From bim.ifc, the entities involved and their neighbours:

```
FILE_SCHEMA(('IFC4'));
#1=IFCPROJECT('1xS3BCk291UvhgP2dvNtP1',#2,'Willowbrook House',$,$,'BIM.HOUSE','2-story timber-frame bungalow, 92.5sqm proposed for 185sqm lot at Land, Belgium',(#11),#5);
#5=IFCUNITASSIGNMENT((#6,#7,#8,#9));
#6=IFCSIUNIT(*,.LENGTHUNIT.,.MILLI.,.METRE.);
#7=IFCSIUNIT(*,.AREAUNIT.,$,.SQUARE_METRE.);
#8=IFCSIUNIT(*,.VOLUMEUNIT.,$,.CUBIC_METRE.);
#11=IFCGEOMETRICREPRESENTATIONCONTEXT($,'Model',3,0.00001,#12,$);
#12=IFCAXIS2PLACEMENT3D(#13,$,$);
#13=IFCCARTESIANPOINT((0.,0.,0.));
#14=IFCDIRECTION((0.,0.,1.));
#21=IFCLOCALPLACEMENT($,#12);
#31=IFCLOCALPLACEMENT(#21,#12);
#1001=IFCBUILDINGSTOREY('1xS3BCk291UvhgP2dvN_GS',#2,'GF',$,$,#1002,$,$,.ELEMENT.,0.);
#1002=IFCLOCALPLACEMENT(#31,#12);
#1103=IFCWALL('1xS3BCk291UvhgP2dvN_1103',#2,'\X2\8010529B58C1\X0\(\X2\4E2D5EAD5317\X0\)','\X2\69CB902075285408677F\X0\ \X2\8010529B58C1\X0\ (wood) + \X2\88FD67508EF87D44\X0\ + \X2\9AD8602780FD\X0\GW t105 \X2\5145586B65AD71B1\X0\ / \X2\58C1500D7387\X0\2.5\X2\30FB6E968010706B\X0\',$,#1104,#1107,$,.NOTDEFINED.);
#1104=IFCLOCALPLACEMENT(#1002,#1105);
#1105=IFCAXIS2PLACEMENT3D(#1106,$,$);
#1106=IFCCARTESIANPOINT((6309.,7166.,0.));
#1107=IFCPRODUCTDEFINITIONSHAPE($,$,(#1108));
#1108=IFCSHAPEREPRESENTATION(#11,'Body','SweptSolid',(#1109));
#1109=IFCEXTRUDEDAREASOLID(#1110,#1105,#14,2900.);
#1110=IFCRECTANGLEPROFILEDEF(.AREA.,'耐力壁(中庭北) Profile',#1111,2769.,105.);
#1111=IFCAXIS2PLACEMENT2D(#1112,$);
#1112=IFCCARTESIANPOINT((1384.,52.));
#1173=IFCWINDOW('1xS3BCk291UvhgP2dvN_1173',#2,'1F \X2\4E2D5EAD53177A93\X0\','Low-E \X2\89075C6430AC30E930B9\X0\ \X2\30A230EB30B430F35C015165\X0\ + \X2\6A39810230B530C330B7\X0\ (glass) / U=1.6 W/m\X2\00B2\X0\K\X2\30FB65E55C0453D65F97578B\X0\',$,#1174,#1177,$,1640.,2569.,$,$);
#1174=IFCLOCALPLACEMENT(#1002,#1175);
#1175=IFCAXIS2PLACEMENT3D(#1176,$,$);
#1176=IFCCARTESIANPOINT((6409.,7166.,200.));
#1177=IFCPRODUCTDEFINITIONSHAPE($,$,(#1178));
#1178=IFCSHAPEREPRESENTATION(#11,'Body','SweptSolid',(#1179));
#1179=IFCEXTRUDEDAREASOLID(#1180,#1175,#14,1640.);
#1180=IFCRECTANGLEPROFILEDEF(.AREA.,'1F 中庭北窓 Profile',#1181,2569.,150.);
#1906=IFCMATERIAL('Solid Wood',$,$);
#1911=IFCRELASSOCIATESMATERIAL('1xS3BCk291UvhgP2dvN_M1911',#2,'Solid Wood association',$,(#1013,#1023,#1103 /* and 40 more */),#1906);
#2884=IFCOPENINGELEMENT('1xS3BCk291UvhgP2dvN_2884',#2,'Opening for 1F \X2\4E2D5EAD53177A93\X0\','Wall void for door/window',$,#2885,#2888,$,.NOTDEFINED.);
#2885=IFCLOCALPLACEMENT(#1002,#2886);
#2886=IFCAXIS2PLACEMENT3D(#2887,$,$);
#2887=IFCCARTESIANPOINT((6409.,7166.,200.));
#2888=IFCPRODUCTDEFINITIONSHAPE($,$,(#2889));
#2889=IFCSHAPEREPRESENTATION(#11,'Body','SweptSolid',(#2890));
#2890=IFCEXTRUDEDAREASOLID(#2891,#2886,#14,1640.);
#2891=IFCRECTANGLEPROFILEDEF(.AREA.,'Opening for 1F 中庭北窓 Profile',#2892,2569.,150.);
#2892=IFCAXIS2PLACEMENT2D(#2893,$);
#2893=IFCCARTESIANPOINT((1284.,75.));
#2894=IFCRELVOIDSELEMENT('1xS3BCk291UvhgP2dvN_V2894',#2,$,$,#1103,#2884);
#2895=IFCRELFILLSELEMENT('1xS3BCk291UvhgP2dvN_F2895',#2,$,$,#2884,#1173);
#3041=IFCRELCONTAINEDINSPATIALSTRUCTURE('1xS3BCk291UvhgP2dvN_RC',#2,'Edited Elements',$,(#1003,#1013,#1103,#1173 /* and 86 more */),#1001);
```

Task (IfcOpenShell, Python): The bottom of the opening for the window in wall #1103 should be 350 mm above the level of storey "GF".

```python
import numpy as np
import ifcopenshell
import ifcopenshell.api.geometry
import ifcopenshell.geom
import ifcopenshell.util.element
import ifcopenshell.util.placement
import ifcopenshell.util.shape
import ifcopenshell.util.unit

model = ifcopenshell.open("bim.ifc")
unit_scale = ifcopenshell.util.unit.calculate_unit_scale(model)

window = model.by_id(1173)
opening = window.FillsVoids[0].RelatingOpeningElement
storey = ifcopenshell.util.element.get_container(window, ifc_class="IfcBuildingStorey")
level = ifcopenshell.util.placement.get_local_placement(storey.ObjectPlacement)[2, 3]

# The opening's origin need not be at the sill, so measure its lowest point.
shape = ifcopenshell.geom.create_shape(ifcopenshell.geom.settings(), opening)
bottom = ifcopenshell.util.shape.get_shape_bottom_elevation(shape, shape.geometry) / unit_scale
dz = level + 350.0 - bottom

shift = np.array([0.0, 0.0, dz])
# The window is not placed relative to its opening, so move both.
for product in (opening, window):
    matrix = ifcopenshell.util.placement.get_local_placement(product.ObjectPlacement)
    matrix[:3, 3] += shift
    ifcopenshell.api.geometry.edit_object_placement(model, product=product, matrix=matrix, is_si=False)

print(f"moved by {dz * unit_scale:+.3f} m")

model.write("bim_updated.ifc")
```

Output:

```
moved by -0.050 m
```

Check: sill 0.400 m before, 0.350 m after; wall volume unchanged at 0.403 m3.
